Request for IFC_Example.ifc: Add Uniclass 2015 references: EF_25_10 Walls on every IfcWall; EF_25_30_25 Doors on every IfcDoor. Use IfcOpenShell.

First a look at what the model holds.

```python
import ifcopenshell

model = ifcopenshell.open("IFC_Example.ifc")
print(model.schema)
print("classifications:", [c.Name for c in model.by_type("IfcClassification")])
for ifc_class in ("IfcDoor", "IfcRoof", "IfcStair", "IfcWall", "IfcWindow"):
    print(ifc_class, len(model.by_type(ifc_class)))
```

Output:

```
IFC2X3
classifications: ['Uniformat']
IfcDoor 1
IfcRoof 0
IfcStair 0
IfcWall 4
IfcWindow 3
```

```python
import ifcopenshell
import ifcopenshell.api.classification

model = ifcopenshell.open("IFC_Example.ifc")

# IFC2X3 requires Source and Edition and has no link from the project to the system.
system = model.create_entity("IfcClassification", Source="NBS", Edition="2015", Name="Uniclass 2015")

codes = {
    "IfcWall": ("EF_25_10", "Walls"),
    "IfcDoor": ("EF_25_30_25", "Doors"),
}
for ifc_class, (code, name) in codes.items():
    products = model.by_type(ifc_class)
    ifcopenshell.api.classification.add_reference(
        model, products=products, classification=system, identification=code, name=name
    )
    print(code, len(products))

model.write("IFC_Example_rev.ifc")
```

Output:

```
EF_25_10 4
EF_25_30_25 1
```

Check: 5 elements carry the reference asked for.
